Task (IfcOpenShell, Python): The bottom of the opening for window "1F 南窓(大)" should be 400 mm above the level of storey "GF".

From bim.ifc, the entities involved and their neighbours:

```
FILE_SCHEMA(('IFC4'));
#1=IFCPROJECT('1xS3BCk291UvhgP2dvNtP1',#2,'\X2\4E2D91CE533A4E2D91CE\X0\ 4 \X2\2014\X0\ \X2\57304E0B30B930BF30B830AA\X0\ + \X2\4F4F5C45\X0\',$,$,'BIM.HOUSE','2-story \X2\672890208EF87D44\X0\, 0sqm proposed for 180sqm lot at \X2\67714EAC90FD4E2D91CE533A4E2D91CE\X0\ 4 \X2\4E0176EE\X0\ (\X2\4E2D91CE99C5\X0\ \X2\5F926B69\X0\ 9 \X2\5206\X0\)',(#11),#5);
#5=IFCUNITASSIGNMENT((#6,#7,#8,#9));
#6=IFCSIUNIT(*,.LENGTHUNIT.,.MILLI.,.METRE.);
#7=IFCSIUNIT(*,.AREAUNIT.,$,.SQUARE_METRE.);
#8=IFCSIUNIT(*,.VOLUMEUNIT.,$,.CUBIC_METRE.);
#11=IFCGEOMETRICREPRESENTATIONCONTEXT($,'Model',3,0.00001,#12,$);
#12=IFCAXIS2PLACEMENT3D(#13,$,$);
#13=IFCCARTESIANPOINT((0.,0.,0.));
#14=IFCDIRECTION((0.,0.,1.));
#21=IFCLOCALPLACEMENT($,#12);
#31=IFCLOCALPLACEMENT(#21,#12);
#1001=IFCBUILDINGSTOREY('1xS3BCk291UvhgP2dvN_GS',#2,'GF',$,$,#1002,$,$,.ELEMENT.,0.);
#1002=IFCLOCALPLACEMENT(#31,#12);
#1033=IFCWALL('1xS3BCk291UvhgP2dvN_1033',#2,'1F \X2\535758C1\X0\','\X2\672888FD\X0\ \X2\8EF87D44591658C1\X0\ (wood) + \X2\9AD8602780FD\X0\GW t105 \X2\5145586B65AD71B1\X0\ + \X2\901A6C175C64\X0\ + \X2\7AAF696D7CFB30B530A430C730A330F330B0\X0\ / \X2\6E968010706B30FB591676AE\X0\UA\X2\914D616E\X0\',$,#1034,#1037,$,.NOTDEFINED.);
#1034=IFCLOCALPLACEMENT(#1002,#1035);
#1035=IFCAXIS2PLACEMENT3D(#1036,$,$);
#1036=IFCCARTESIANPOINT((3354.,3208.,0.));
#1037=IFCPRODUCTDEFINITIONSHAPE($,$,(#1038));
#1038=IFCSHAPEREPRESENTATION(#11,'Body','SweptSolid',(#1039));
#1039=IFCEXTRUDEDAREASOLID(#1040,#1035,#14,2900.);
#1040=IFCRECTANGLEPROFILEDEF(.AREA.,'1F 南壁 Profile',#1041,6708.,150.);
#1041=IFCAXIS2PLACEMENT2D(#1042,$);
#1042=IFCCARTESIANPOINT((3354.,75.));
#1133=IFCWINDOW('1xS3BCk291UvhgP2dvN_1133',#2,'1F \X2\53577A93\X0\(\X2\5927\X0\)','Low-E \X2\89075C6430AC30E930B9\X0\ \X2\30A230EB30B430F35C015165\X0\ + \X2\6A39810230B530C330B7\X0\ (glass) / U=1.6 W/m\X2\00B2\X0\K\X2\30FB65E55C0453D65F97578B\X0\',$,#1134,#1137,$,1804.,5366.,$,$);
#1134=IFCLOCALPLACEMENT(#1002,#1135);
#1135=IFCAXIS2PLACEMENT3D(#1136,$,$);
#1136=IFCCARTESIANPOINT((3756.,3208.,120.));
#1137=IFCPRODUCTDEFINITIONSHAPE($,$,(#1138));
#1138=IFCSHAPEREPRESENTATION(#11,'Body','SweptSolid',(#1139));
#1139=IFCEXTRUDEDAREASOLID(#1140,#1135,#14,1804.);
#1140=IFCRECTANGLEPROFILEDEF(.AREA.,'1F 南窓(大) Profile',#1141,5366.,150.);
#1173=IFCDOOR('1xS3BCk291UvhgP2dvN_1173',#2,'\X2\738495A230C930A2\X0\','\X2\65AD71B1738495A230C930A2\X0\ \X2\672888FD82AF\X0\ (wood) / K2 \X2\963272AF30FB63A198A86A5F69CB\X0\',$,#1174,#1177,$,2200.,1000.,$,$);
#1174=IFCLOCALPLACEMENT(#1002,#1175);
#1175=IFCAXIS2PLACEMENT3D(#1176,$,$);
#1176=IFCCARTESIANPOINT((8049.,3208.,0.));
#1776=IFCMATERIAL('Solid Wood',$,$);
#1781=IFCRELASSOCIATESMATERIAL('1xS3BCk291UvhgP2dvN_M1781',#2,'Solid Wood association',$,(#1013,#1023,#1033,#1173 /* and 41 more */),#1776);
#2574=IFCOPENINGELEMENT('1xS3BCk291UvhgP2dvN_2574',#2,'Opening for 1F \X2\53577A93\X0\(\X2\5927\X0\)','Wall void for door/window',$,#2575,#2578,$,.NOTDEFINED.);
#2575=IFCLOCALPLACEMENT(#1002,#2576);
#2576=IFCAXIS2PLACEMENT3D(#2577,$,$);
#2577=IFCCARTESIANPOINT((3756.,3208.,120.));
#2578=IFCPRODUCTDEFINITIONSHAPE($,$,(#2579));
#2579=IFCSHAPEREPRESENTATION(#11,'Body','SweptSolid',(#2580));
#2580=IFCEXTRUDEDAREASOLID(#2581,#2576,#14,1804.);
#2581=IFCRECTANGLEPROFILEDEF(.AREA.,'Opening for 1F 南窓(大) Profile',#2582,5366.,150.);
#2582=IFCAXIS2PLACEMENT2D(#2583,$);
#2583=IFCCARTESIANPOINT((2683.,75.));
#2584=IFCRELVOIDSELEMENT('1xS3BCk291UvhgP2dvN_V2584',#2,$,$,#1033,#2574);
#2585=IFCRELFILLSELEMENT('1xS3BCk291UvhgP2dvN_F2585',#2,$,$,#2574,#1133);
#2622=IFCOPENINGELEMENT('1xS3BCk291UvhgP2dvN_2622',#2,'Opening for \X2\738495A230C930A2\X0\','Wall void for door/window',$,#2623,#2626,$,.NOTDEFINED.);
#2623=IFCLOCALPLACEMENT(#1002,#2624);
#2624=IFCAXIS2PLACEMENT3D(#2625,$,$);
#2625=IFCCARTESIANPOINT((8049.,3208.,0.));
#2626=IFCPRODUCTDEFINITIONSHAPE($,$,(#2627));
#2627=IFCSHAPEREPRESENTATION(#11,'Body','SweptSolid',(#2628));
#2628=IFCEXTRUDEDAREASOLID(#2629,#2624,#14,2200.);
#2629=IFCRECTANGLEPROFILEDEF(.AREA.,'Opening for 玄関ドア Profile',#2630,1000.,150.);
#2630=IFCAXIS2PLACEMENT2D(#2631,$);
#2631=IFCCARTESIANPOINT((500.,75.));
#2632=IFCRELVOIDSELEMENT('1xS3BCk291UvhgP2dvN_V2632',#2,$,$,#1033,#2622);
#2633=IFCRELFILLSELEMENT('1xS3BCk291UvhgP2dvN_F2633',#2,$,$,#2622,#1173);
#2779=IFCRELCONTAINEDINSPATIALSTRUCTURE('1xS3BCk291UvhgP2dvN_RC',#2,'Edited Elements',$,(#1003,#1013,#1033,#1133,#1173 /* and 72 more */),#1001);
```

```python
import numpy as np
import ifcopenshell
import ifcopenshell.api.geometry
import ifcopenshell.geom
import ifcopenshell.util.element
import ifcopenshell.util.placement
import ifcopenshell.util.shape
import ifcopenshell.util.unit

model = ifcopenshell.open("bim.ifc")
unit_scale = ifcopenshell.util.unit.calculate_unit_scale(model)

window = model.by_guid("1xS3BCk291UvhgP2dvN_1133")
opening = window.FillsVoids[0].RelatingOpeningElement
storey = ifcopenshell.util.element.get_container(window, ifc_class="IfcBuildingStorey")
level = ifcopenshell.util.placement.get_local_placement(storey.ObjectPlacement)[2, 3]

# The opening's origin need not be at the sill, so measure its lowest point.
shape = ifcopenshell.geom.create_shape(ifcopenshell.geom.settings(), opening)
bottom = ifcopenshell.util.shape.get_shape_bottom_elevation(shape, shape.geometry) / unit_scale
dz = level + 0.4 / unit_scale - bottom

shift = np.array([0.0, 0.0, dz])
# The window is not placed relative to its opening, so move both.
for product in (opening, window):
    matrix = ifcopenshell.util.placement.get_local_placement(product.ObjectPlacement)
    matrix[:3, 3] += shift
    ifcopenshell.api.geometry.edit_object_placement(model, product=product, matrix=matrix, is_si=False)

print(f"moved by {dz * unit_scale:+.3f} m")

model.write("bim_v2.ifc")
```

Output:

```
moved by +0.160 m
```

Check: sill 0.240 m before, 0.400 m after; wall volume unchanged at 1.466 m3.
